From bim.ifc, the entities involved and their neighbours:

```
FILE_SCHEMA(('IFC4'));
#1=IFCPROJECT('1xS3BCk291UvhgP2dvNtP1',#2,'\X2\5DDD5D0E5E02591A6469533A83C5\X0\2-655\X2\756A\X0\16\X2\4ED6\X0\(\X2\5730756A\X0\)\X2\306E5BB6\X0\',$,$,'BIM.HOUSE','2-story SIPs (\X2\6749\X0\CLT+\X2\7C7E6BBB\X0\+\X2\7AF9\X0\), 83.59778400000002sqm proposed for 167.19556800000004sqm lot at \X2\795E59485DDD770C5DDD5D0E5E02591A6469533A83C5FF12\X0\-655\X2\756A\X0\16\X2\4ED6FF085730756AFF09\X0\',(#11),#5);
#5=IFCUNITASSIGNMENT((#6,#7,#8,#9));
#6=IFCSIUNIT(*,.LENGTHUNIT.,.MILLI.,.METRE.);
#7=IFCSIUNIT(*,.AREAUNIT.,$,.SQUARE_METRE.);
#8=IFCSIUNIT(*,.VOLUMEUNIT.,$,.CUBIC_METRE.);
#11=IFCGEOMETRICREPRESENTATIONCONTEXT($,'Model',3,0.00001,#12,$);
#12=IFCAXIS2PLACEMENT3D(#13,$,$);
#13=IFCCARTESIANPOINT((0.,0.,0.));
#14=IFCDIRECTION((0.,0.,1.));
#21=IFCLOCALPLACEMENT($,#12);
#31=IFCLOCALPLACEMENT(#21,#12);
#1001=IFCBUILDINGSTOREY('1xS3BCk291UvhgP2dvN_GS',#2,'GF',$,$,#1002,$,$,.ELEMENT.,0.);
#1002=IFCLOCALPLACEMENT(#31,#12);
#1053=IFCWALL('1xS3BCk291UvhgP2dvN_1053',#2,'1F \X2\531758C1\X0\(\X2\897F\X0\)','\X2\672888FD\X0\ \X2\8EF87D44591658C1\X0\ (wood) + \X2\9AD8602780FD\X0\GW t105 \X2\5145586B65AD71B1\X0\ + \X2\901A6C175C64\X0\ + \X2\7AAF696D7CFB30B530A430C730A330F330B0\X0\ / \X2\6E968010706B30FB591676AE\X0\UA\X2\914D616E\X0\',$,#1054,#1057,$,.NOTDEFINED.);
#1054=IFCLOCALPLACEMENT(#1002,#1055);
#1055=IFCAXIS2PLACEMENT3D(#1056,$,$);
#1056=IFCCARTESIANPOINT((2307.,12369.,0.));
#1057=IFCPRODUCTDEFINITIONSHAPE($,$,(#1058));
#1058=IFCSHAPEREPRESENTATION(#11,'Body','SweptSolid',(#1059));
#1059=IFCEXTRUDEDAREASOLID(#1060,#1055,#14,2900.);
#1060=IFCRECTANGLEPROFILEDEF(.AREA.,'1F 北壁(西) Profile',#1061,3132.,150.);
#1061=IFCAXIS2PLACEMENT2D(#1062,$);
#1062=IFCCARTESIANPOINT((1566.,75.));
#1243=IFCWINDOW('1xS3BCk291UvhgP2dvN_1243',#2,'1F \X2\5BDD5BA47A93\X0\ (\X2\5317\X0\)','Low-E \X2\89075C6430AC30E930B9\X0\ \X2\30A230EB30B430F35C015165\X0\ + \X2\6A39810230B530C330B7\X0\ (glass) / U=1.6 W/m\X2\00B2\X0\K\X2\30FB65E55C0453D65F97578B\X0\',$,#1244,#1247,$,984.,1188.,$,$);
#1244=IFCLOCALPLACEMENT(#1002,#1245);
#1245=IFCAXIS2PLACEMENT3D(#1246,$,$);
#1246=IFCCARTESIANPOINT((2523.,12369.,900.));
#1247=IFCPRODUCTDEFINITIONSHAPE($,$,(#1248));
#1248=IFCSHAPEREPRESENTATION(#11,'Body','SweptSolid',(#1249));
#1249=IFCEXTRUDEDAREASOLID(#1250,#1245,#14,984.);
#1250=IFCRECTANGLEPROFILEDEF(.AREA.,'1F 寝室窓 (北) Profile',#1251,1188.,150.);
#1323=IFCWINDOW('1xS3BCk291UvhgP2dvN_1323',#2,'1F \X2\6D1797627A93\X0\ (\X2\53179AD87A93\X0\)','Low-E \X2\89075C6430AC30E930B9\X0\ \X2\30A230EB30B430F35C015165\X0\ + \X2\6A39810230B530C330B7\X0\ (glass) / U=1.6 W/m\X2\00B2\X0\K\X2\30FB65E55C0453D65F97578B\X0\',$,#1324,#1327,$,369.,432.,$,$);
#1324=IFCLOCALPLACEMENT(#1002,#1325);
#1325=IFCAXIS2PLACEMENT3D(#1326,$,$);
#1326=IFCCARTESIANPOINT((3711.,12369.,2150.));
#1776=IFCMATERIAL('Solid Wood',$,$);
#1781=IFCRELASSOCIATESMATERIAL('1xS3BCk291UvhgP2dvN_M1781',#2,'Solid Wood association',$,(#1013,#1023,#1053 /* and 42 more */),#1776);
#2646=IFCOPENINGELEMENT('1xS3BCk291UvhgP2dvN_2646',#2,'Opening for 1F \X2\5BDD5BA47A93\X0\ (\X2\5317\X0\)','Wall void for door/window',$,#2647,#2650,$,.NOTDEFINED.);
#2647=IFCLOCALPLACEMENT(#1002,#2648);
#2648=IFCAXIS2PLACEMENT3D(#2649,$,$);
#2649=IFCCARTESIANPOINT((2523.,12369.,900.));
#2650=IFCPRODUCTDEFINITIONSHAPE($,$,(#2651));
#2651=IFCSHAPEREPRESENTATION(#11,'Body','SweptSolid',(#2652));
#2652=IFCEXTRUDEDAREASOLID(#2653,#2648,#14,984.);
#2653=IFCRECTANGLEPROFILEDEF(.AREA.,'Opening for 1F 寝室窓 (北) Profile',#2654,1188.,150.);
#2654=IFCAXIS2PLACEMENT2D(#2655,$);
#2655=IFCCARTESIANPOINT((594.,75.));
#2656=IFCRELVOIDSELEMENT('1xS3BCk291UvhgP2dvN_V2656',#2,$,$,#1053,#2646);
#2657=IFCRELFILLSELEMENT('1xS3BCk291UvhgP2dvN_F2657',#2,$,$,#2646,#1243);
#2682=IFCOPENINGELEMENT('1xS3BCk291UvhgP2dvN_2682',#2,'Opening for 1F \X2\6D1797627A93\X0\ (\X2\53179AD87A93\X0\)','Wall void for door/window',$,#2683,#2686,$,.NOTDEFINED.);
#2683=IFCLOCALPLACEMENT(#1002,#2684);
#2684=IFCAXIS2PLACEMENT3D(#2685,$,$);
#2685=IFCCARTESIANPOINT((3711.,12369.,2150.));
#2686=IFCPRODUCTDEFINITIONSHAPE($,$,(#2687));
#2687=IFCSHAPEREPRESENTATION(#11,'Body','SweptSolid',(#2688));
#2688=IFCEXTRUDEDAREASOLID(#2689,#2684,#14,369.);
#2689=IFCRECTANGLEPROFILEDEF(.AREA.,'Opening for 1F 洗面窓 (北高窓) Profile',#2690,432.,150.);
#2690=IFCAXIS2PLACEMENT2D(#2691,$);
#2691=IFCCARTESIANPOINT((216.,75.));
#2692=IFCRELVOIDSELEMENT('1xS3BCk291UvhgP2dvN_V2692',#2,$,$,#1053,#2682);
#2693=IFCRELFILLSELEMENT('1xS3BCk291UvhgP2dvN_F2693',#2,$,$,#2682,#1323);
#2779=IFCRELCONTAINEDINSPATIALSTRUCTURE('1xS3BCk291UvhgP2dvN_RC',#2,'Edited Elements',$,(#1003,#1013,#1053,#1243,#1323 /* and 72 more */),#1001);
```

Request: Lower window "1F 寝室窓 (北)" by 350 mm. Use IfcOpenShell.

```python
import numpy as np
import ifcopenshell
import ifcopenshell.api.geometry
import ifcopenshell.util.placement
import ifcopenshell.util.unit

model = ifcopenshell.open("bim.ifc")
unit_scale = ifcopenshell.util.unit.calculate_unit_scale(model)

window = model.by_guid("1xS3BCk291UvhgP2dvN_1243")
opening = window.FillsVoids[0].RelatingOpeningElement
dz = -0.35 / unit_scale

shift = np.array([0.0, 0.0, dz])
# The window is not placed relative to its opening, so move both.
for product in (opening, window):
    matrix = ifcopenshell.util.placement.get_local_placement(product.ObjectPlacement)
    matrix[:3, 3] += shift
    ifcopenshell.api.geometry.edit_object_placement(model, product=product, matrix=matrix, is_si=False)

print(f"moved by {dz * unit_scale:+.3f} m")

model.write("bim-out.ifc")
```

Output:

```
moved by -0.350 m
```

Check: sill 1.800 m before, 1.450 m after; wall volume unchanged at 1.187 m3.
